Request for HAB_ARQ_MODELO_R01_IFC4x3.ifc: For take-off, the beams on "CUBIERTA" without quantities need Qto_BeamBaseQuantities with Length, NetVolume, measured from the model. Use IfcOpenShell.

First a look at what the model holds.

```python
import ifcopenshell
import ifcopenshell.util.element
import ifcopenshell.util.unit

model = ifcopenshell.open("HAB_ARQ_MODELO_R01_IFC4x3.ifc")
print(model.schema)
for unit_type in ("LENGTHUNIT", "AREAUNIT", "VOLUMEUNIT"):
    print(unit_type, ifcopenshell.util.unit.calculate_unit_scale(model, unit_type))
storey = next(s for s in model.by_type("IfcBuildingStorey") if s.Name == "CUBIERTA")
beams = [e for e in ifcopenshell.util.element.get_decomposition(storey) if e.is_a("IfcBeam")]
for e in sorted(beams, key=lambda e: e.id()):
    print(e.id(), e.is_a(), e.Name, list(ifcopenshell.util.element.get_psets(e, qtos_only=True)), sep=" | ")
```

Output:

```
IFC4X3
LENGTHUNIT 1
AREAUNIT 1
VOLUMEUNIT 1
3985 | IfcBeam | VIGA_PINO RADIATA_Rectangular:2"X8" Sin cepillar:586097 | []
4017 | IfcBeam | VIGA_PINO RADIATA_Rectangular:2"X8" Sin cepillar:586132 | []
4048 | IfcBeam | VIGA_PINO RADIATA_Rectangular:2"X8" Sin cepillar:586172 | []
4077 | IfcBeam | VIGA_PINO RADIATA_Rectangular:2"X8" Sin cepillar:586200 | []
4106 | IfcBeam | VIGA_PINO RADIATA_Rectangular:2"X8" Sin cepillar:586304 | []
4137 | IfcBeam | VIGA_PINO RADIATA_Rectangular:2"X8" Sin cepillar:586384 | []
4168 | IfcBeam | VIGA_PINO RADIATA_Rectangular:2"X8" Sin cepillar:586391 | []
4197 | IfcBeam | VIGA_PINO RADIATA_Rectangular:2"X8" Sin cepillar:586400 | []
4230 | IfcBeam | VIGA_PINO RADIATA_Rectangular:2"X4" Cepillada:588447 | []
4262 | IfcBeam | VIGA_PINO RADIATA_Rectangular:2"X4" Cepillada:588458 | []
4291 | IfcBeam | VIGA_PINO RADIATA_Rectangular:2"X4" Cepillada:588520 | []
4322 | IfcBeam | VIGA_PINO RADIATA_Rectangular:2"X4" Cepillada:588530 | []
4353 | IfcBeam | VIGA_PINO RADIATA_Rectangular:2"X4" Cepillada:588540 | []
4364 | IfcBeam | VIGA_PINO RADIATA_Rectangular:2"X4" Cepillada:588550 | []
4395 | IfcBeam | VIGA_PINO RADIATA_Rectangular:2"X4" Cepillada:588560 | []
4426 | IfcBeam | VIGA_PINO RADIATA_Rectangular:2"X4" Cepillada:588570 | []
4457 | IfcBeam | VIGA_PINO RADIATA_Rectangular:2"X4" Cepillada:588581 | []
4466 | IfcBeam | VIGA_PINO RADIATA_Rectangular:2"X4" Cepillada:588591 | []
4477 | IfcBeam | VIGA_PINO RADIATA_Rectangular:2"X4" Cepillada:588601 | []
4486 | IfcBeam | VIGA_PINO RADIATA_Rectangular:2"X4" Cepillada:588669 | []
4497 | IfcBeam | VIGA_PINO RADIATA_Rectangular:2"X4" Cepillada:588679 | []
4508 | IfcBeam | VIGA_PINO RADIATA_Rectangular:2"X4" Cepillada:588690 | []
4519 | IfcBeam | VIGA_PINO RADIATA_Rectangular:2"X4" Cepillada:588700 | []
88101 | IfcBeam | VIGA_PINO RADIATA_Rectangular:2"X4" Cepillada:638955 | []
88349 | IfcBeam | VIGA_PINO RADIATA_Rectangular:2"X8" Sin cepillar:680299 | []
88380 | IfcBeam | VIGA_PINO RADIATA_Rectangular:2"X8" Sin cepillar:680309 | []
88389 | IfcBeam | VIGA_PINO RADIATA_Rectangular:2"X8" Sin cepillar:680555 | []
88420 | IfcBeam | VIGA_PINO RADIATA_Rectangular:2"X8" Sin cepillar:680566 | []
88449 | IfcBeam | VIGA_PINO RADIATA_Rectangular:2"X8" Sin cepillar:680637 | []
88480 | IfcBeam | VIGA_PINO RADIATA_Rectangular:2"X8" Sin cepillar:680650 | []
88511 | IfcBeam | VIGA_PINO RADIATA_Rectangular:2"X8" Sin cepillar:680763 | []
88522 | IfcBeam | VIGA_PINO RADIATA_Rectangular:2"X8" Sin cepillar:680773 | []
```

```python
import ifcopenshell
import ifcopenshell.api.pset
import ifcopenshell.geom
import ifcopenshell.util.element
import ifcopenshell.util.shape
import ifcopenshell.util.unit

model = ifcopenshell.open("HAB_ARQ_MODELO_R01_IFC4x3.ifc")
unit_scale = ifcopenshell.util.unit.calculate_unit_scale(model)
volume_scale = ifcopenshell.util.unit.calculate_unit_scale(model, "VOLUMEUNIT")
settings = ifcopenshell.geom.settings()

storey = next(s for s in model.by_type("IfcBuildingStorey") if s.Name == "CUBIERTA")
beams = [e for e in ifcopenshell.util.element.get_decomposition(storey) if e.is_a("IfcBeam")]

for e in sorted(beams, key=lambda e: e.id()):
    if ifcopenshell.util.element.get_psets(e, qtos_only=True, should_inherit=False):
        continue
    # Geometry comes back in metres, in the element's own axes.
    shape = ifcopenshell.geom.create_shape(settings, e)
    values = {
        "Length": ifcopenshell.util.shape.get_max_xyz(shape.geometry) / unit_scale,
        "NetVolume": ifcopenshell.util.shape.get_volume(shape.geometry) / volume_scale,
    }
    qto = ifcopenshell.api.pset.add_qto(model, product=e, name="Qto_BeamBaseQuantities")
    ifcopenshell.api.pset.edit_qto(model, qto=qto, properties=values)
    print(e.id(), {k: round(v, 3) for k, v in values.items()})

model.write("HAB_ARQ_MODELO_R01_IFC4x3_updated.ifc")
```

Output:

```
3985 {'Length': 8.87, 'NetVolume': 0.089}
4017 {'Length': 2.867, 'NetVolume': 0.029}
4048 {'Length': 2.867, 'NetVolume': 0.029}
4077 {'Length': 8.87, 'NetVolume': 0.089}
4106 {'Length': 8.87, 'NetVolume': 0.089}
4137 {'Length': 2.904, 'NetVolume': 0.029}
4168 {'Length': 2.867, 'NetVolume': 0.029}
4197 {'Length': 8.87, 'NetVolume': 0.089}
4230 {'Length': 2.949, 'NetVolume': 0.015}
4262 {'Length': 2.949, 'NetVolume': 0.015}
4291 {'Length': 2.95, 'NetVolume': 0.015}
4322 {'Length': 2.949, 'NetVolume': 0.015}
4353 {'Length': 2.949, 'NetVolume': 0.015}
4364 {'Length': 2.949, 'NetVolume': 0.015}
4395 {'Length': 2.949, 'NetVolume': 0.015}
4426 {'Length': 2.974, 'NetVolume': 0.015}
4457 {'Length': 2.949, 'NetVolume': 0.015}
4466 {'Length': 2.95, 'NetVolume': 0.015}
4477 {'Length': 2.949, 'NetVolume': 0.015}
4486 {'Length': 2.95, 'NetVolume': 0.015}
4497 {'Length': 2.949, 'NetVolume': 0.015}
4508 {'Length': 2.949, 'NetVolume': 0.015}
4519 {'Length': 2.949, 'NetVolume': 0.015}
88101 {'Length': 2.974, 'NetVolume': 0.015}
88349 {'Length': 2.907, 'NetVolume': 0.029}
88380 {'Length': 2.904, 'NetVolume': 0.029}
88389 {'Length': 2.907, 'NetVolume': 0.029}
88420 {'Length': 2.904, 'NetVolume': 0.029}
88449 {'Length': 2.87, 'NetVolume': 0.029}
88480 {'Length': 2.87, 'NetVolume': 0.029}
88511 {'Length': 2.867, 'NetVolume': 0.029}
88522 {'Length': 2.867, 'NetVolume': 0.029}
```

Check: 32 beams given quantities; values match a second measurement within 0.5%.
